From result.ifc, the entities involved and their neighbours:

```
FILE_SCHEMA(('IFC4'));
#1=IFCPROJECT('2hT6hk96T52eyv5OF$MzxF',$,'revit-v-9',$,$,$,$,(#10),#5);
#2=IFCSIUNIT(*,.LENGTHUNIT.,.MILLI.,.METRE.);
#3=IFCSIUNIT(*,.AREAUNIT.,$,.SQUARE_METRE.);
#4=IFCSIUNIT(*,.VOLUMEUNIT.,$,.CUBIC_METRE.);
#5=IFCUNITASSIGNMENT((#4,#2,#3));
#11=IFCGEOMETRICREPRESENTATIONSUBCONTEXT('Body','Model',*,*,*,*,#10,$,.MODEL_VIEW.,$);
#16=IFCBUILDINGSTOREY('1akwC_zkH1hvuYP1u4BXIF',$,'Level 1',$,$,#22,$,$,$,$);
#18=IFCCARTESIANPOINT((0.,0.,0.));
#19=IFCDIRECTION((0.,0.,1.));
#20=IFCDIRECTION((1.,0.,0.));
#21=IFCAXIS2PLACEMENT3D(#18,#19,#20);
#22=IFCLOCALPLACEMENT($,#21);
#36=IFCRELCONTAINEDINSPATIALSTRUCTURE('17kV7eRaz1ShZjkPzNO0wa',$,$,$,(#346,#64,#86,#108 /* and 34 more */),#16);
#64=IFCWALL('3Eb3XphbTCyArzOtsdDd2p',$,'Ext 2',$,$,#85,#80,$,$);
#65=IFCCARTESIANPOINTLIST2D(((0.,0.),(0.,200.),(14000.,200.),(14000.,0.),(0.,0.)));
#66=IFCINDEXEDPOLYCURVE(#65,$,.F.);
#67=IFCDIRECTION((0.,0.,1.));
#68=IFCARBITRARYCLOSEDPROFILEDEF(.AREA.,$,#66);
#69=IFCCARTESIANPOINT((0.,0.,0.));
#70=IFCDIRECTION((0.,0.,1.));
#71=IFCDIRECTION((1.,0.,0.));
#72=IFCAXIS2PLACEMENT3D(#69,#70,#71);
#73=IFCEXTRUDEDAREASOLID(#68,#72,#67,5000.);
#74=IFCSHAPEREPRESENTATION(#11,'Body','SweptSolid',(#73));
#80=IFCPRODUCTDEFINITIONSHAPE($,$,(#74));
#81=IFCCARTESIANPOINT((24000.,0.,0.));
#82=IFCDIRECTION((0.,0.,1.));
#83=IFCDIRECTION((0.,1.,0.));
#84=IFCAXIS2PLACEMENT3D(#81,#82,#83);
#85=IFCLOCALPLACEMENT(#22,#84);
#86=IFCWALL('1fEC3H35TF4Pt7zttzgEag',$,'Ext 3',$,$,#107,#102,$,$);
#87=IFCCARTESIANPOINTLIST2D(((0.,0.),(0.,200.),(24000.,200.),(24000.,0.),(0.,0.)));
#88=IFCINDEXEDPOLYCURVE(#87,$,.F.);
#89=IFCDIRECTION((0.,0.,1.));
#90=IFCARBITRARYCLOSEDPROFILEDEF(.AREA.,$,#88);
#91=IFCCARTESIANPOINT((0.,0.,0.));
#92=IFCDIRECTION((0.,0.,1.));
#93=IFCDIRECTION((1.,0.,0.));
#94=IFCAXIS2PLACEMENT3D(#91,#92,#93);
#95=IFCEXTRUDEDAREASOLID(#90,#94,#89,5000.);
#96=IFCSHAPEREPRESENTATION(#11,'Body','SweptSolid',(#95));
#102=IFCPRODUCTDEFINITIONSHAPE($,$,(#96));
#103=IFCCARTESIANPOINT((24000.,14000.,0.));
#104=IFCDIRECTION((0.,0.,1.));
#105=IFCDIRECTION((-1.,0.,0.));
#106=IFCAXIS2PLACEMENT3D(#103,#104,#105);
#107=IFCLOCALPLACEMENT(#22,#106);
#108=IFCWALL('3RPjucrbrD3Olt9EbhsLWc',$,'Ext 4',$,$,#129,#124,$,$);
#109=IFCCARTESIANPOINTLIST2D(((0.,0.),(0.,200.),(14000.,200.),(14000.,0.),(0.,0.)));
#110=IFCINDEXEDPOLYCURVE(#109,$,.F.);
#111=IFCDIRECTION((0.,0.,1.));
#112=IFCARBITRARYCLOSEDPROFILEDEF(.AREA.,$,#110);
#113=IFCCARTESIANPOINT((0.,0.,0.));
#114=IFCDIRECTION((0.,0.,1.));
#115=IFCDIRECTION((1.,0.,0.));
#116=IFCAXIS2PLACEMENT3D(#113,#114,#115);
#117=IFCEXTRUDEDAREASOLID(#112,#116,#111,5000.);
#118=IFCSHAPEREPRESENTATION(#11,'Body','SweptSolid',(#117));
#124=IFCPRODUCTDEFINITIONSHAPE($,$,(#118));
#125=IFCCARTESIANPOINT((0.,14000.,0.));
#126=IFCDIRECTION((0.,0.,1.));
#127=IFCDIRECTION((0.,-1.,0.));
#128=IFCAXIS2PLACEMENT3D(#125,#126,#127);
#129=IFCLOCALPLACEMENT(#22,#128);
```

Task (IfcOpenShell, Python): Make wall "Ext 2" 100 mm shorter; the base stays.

```python
import ifcopenshell
import ifcopenshell.geom
import ifcopenshell.util.representation
import ifcopenshell.util.shape
import ifcopenshell.util.unit

model = ifcopenshell.open("result.ifc")
unit_scale = ifcopenshell.util.unit.calculate_unit_scale(model)
settings = ifcopenshell.geom.settings()


def volume(element):
    """Net volume in cubic metres, openings subtracted."""
    shape = ifcopenshell.geom.create_shape(settings, element)
    return ifcopenshell.util.shape.get_volume(shape.geometry)


wall = model.by_guid("3Eb3XphbTCyArzOtsdDd2p")
before = volume(wall)

body = ifcopenshell.util.representation.get_representation(wall, "Model", "Body")
solid = body.Items[0]
old_height = solid.Depth
solid.Depth -= 0.1 / unit_scale
after = volume(wall)

print(f"height {old_height:g} -> {solid.Depth:g}, volume {before:.3f} -> {after:.3f} m3")

model.write("result_v2.ifc")
```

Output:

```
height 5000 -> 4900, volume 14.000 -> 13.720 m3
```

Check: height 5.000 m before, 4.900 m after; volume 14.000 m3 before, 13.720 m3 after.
